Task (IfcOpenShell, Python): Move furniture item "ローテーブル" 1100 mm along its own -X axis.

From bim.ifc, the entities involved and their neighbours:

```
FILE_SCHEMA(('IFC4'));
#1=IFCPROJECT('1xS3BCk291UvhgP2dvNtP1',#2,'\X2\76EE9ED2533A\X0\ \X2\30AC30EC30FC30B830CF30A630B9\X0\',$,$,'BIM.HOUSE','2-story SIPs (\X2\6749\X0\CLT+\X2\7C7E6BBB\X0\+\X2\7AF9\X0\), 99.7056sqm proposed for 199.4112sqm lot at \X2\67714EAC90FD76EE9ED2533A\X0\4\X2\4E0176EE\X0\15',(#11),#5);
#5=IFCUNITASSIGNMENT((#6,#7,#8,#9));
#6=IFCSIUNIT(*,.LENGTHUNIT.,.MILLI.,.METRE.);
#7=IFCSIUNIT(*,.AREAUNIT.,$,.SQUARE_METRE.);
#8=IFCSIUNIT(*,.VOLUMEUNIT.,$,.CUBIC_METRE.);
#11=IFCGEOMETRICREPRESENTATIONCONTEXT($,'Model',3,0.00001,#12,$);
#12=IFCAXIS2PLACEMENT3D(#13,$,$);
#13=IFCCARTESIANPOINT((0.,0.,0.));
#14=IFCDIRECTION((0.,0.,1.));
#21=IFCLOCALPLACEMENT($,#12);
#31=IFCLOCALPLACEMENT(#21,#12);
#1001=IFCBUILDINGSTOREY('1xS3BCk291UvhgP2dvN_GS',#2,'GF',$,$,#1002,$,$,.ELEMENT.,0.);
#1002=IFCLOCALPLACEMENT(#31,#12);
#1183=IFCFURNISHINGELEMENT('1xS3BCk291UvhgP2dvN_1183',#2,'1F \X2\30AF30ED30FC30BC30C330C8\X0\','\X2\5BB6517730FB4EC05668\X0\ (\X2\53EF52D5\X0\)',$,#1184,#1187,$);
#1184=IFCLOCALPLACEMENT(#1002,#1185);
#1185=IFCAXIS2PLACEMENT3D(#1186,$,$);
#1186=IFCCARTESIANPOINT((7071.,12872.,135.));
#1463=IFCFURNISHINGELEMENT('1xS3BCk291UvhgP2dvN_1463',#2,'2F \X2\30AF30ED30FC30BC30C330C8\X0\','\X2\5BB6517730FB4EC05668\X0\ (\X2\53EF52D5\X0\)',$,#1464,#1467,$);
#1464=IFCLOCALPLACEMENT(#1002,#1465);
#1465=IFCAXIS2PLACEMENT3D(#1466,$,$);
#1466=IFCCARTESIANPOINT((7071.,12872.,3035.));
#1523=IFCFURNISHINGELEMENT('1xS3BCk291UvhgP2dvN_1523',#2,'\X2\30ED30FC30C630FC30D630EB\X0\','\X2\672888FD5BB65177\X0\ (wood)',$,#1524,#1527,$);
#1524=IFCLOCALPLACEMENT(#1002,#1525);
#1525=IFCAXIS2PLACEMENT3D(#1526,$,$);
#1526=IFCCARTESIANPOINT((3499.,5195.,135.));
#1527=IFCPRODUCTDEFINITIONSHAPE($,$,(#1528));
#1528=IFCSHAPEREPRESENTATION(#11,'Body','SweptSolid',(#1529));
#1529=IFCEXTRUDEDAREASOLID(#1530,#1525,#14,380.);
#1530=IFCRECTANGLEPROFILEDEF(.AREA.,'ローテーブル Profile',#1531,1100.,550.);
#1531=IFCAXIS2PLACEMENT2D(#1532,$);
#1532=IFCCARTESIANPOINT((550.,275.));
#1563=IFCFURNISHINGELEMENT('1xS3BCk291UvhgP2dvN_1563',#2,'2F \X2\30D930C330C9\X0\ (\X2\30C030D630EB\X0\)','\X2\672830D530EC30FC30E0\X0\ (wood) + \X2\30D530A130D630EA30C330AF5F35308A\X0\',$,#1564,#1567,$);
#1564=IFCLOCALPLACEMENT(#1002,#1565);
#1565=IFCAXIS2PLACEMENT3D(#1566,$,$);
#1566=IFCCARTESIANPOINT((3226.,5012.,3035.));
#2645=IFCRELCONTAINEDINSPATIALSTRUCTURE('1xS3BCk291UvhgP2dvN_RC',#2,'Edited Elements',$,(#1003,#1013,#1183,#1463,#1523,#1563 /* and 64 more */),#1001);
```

```python
import ifcopenshell
import ifcopenshell.api.geometry
import ifcopenshell.util.placement

model = ifcopenshell.open("bim.ifc")

item = model.by_id(1523)
matrix = ifcopenshell.util.placement.get_local_placement(item.ObjectPlacement)
matrix[:3, 3] -= matrix[:3, 0] * 1100.0
ifcopenshell.api.geometry.edit_object_placement(model, product=item, matrix=matrix, is_si=False)

print(ifcopenshell.util.placement.get_local_placement(item.ObjectPlacement).round(3) + 0.0)

model.write("bim_rev.ifc")
```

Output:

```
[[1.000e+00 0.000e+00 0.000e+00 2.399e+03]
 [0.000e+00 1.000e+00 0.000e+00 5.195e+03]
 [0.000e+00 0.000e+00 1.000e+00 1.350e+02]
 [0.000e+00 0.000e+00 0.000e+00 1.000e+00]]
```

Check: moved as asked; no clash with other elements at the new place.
